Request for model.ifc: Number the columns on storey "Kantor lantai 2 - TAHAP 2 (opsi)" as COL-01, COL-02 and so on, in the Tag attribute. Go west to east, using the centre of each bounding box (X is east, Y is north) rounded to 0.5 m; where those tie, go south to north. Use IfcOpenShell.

First a look at what the model holds.

```python
import ifcopenshell
import ifcopenshell.util.element
import ifcopenshell.util.placement

model = ifcopenshell.open("model.ifc")
print(model.schema)
storey = next(s for s in model.by_type("IfcBuildingStorey") if s.Name == "Kantor lantai 2 - TAHAP 2 (opsi)")
columns = [e for e in ifcopenshell.util.element.get_decomposition(storey) if e.is_a("IfcColumn")]
for e in sorted(columns, key=lambda e: e.id()):
    origin = ifcopenshell.util.placement.get_local_placement(e.ObjectPlacement)[:3, 3]
    print(e.id(), e.Tag, e.Name, origin.round(2) + 0.0, sep=" | ")
```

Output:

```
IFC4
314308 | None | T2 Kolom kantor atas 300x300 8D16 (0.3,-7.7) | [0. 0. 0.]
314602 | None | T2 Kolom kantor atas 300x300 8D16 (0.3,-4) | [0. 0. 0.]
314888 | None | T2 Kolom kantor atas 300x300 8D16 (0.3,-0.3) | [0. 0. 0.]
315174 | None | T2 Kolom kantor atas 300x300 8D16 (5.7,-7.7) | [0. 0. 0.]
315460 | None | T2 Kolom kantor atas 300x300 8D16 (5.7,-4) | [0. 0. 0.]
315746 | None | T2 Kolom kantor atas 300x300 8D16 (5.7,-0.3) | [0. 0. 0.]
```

```python
import ifcopenshell
import ifcopenshell.geom
import ifcopenshell.util.element
import ifcopenshell.util.shape

model = ifcopenshell.open("model.ifc")
settings = ifcopenshell.geom.settings()
settings.set("use-world-coords", True)


def centre(element):
    shape = ifcopenshell.geom.create_shape(settings, element)
    return ifcopenshell.util.shape.get_bbox_centroid(shape.geometry)


storey = next(s for s in model.by_type("IfcBuildingStorey") if s.Name == "Kantor lantai 2 - TAHAP 2 (opsi)")
columns = [e for e in ifcopenshell.util.element.get_decomposition(storey) if e.is_a("IfcColumn")]

# Insertion points can sit at a corner or the storey origin, so sort by the geometry (in metres).
centres = {e: centre(e) for e in columns}
columns.sort(key=lambda e: (round(centres[e][0] / 0.5), centres[e][1]))

for i, e in enumerate(columns, start=1):
    number = f"COL-{i:02d}"
    e.Tag = number
    print(e.id(), number)

model.write("model_rev.ifc")
```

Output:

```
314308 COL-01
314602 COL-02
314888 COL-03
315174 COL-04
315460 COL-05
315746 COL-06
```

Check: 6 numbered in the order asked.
